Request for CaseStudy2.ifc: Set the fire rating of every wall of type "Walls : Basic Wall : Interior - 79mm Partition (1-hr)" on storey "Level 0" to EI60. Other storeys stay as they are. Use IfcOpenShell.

First a look at what the model holds.

```python
import ifcopenshell
import ifcopenshell.util.element

model = ifcopenshell.open("CaseStudy2.ifc")
print(model.schema)
storey = next(s for s in model.by_type("IfcBuildingStorey") if s.Name == "Level 0")
walls = [e for e in ifcopenshell.util.element.get_decomposition(storey) if e.is_a("IfcWall")]
seen = {}
for e in walls:
    element_type = ifcopenshell.util.element.get_type(e)
    key = (element_type.Name if element_type != e and element_type else None, ifcopenshell.util.element.get_pset(e, "Pset_WallCommon", "FireRating"))
    seen[key] = seen.get(key, 0) + 1
for (name, value), count in sorted(seen.items(), key=str):
    print(count, "x", name, "|", value)
```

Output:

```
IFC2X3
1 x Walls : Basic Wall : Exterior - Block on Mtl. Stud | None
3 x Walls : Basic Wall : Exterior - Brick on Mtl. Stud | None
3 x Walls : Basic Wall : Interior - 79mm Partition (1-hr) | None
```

```python
import ifcopenshell
import ifcopenshell.api.pset
import ifcopenshell.util.element

model = ifcopenshell.open("CaseStudy2.ifc")

storey = next(s for s in model.by_type("IfcBuildingStorey") if s.Name == "Level 0")
walls = [e for e in ifcopenshell.util.element.get_decomposition(storey) if e.is_a("IfcWall")]

count = 0
for e in walls:
    element_type = ifcopenshell.util.element.get_type(e)
    if element_type in (None, e) or element_type.Name != "Walls : Basic Wall : Interior - 79mm Partition (1-hr)":
        continue
    # add_pset returns the element's existing set when there is one.
    pset = ifcopenshell.api.pset.add_pset(model, product=e, name="Pset_WallCommon")
    ifcopenshell.api.pset.edit_pset(model, pset=pset, properties={"FireRating": "EI60"})
    count += 1

print(count, "walls updated")

model.write("CaseStudy2_updated.ifc")
```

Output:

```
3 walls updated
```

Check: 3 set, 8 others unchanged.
